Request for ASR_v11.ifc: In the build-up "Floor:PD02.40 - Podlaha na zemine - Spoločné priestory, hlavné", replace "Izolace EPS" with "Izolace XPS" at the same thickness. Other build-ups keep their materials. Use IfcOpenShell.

First a look at what the model holds.

```python
import ifcopenshell
import ifcopenshell.util.element

model = ifcopenshell.open("ASR_v11.ifc")
print(model.schema)
for layer_set in model.by_type("IfcMaterialLayerSet"):
    if layer_set.LayerSetName == "Floor:PD02.40 - Podlaha na zemine - Spoločné priestory, hlavné":
        for layer in layer_set.MaterialLayers:
            print(layer.id(), layer.Material and layer.Material.Name, layer.LayerThickness, sep=" | ")
        print(len(ifcopenshell.util.element.get_elements_by_material(model, layer_set)), "elements and types use it")
print(sorted(m.Name for m in model.by_type("IfcMaterial") if m.Name)[:60])
```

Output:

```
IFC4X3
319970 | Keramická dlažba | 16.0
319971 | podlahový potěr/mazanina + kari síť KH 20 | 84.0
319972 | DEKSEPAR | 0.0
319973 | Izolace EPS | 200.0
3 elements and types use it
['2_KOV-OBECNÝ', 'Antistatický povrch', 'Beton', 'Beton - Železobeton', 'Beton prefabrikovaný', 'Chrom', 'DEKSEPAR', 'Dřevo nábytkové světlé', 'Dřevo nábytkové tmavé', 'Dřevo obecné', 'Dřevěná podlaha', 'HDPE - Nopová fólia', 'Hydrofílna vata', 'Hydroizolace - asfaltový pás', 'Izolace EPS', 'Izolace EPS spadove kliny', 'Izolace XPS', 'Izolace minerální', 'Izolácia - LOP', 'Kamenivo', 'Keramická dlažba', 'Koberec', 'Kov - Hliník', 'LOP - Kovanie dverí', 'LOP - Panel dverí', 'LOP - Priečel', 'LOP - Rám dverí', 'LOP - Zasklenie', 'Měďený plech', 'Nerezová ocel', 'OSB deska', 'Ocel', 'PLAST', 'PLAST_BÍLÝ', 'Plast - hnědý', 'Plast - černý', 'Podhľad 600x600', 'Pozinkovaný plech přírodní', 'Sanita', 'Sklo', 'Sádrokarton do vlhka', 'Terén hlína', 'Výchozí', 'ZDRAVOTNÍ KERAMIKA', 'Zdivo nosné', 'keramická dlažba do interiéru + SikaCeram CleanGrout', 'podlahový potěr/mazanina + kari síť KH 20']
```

```python
import ifcopenshell
import ifcopenshell.api.material

model = ifcopenshell.open("ASR_v11.ifc")

layer_set = next(s for s in model.by_type("IfcMaterialLayerSet") if s.LayerSetName == "Floor:PD02.40 - Podlaha na zemine - Spoločné priestory, hlavné")
layer = next(l for l in layer_set.MaterialLayers if l.Material and l.Material.Name == "Izolace EPS")
material = next(m for m in model.by_type("IfcMaterial") if m.Name == "Izolace XPS")

# Point this one layer at the other material; renaming the old one would change it everywhere.
ifcopenshell.api.material.edit_layer(model, layer=layer, attributes={"Name": material.Name}, material=material)

print([l.Material.Name if l.Material else None for l in layer_set.MaterialLayers])

model.write("ASR_v11-out.ifc")
```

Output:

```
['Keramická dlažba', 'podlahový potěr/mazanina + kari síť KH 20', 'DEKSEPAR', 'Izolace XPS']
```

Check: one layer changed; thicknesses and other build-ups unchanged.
